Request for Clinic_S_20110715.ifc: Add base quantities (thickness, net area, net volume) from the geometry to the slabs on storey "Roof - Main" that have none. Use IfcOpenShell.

First a look at what the model holds.

```python
import ifcopenshell
import ifcopenshell.util.element
import ifcopenshell.util.unit

model = ifcopenshell.open("Clinic_S_20110715.ifc")
print(model.schema)
for unit_type in ("LENGTHUNIT", "AREAUNIT", "VOLUMEUNIT"):
    print(unit_type, ifcopenshell.util.unit.calculate_unit_scale(model, unit_type))
storey = next(s for s in model.by_type("IfcBuildingStorey") if s.Name == "Roof - Main")
slabs = [e for e in ifcopenshell.util.element.get_decomposition(storey) if e.is_a("IfcSlab")]
for e in sorted(slabs, key=lambda e: e.id()):
    print(e.id(), e.is_a(), e.Name, list(ifcopenshell.util.element.get_psets(e, qtos_only=True)), sep=" | ")
```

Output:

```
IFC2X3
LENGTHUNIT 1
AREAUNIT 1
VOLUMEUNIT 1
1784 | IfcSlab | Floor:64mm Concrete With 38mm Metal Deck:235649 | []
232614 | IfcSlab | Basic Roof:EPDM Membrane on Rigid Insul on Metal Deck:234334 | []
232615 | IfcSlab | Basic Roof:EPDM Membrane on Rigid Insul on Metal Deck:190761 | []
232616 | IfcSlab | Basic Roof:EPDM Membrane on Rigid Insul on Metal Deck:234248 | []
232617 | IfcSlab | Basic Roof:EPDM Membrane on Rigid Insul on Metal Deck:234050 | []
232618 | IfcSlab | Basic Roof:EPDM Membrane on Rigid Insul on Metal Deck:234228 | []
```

```python
import ifcopenshell
import ifcopenshell.api.pset
import ifcopenshell.geom
import ifcopenshell.util.element
import ifcopenshell.util.shape
import ifcopenshell.util.unit

model = ifcopenshell.open("Clinic_S_20110715.ifc")
unit_scale = ifcopenshell.util.unit.calculate_unit_scale(model)
area_scale = ifcopenshell.util.unit.calculate_unit_scale(model, "AREAUNIT")
volume_scale = ifcopenshell.util.unit.calculate_unit_scale(model, "VOLUMEUNIT")
settings = ifcopenshell.geom.settings()

storey = next(s for s in model.by_type("IfcBuildingStorey") if s.Name == "Roof - Main")
slabs = [e for e in ifcopenshell.util.element.get_decomposition(storey) if e.is_a("IfcSlab")]

for e in sorted(slabs, key=lambda e: e.id()):
    if ifcopenshell.util.element.get_psets(e, qtos_only=True, should_inherit=False):
        continue
    # Geometry comes back in metres, in the element's own axes.
    shape = ifcopenshell.geom.create_shape(settings, e)
    values = {
        "Width": ifcopenshell.util.shape.get_z(shape.geometry) / unit_scale,
        "NetArea": ifcopenshell.util.shape.get_footprint_area(shape.geometry) / area_scale,
        "NetVolume": ifcopenshell.util.shape.get_volume(shape.geometry) / volume_scale,
    }
    qto = ifcopenshell.api.pset.add_qto(model, product=e, name="BaseQuantities")
    ifcopenshell.api.pset.edit_qto(model, qto=qto, properties=values)
    print(e.id(), {k: round(v, 3) for k, v in values.items()})

model.write("Clinic_S_20110715_updated.ifc")
```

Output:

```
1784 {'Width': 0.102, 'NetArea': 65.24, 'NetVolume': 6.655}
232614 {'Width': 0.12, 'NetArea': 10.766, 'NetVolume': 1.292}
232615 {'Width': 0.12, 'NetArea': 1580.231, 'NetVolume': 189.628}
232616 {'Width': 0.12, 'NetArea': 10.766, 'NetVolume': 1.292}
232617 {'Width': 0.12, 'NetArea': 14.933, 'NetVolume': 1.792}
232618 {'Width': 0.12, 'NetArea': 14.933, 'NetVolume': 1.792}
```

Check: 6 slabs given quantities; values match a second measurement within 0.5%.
